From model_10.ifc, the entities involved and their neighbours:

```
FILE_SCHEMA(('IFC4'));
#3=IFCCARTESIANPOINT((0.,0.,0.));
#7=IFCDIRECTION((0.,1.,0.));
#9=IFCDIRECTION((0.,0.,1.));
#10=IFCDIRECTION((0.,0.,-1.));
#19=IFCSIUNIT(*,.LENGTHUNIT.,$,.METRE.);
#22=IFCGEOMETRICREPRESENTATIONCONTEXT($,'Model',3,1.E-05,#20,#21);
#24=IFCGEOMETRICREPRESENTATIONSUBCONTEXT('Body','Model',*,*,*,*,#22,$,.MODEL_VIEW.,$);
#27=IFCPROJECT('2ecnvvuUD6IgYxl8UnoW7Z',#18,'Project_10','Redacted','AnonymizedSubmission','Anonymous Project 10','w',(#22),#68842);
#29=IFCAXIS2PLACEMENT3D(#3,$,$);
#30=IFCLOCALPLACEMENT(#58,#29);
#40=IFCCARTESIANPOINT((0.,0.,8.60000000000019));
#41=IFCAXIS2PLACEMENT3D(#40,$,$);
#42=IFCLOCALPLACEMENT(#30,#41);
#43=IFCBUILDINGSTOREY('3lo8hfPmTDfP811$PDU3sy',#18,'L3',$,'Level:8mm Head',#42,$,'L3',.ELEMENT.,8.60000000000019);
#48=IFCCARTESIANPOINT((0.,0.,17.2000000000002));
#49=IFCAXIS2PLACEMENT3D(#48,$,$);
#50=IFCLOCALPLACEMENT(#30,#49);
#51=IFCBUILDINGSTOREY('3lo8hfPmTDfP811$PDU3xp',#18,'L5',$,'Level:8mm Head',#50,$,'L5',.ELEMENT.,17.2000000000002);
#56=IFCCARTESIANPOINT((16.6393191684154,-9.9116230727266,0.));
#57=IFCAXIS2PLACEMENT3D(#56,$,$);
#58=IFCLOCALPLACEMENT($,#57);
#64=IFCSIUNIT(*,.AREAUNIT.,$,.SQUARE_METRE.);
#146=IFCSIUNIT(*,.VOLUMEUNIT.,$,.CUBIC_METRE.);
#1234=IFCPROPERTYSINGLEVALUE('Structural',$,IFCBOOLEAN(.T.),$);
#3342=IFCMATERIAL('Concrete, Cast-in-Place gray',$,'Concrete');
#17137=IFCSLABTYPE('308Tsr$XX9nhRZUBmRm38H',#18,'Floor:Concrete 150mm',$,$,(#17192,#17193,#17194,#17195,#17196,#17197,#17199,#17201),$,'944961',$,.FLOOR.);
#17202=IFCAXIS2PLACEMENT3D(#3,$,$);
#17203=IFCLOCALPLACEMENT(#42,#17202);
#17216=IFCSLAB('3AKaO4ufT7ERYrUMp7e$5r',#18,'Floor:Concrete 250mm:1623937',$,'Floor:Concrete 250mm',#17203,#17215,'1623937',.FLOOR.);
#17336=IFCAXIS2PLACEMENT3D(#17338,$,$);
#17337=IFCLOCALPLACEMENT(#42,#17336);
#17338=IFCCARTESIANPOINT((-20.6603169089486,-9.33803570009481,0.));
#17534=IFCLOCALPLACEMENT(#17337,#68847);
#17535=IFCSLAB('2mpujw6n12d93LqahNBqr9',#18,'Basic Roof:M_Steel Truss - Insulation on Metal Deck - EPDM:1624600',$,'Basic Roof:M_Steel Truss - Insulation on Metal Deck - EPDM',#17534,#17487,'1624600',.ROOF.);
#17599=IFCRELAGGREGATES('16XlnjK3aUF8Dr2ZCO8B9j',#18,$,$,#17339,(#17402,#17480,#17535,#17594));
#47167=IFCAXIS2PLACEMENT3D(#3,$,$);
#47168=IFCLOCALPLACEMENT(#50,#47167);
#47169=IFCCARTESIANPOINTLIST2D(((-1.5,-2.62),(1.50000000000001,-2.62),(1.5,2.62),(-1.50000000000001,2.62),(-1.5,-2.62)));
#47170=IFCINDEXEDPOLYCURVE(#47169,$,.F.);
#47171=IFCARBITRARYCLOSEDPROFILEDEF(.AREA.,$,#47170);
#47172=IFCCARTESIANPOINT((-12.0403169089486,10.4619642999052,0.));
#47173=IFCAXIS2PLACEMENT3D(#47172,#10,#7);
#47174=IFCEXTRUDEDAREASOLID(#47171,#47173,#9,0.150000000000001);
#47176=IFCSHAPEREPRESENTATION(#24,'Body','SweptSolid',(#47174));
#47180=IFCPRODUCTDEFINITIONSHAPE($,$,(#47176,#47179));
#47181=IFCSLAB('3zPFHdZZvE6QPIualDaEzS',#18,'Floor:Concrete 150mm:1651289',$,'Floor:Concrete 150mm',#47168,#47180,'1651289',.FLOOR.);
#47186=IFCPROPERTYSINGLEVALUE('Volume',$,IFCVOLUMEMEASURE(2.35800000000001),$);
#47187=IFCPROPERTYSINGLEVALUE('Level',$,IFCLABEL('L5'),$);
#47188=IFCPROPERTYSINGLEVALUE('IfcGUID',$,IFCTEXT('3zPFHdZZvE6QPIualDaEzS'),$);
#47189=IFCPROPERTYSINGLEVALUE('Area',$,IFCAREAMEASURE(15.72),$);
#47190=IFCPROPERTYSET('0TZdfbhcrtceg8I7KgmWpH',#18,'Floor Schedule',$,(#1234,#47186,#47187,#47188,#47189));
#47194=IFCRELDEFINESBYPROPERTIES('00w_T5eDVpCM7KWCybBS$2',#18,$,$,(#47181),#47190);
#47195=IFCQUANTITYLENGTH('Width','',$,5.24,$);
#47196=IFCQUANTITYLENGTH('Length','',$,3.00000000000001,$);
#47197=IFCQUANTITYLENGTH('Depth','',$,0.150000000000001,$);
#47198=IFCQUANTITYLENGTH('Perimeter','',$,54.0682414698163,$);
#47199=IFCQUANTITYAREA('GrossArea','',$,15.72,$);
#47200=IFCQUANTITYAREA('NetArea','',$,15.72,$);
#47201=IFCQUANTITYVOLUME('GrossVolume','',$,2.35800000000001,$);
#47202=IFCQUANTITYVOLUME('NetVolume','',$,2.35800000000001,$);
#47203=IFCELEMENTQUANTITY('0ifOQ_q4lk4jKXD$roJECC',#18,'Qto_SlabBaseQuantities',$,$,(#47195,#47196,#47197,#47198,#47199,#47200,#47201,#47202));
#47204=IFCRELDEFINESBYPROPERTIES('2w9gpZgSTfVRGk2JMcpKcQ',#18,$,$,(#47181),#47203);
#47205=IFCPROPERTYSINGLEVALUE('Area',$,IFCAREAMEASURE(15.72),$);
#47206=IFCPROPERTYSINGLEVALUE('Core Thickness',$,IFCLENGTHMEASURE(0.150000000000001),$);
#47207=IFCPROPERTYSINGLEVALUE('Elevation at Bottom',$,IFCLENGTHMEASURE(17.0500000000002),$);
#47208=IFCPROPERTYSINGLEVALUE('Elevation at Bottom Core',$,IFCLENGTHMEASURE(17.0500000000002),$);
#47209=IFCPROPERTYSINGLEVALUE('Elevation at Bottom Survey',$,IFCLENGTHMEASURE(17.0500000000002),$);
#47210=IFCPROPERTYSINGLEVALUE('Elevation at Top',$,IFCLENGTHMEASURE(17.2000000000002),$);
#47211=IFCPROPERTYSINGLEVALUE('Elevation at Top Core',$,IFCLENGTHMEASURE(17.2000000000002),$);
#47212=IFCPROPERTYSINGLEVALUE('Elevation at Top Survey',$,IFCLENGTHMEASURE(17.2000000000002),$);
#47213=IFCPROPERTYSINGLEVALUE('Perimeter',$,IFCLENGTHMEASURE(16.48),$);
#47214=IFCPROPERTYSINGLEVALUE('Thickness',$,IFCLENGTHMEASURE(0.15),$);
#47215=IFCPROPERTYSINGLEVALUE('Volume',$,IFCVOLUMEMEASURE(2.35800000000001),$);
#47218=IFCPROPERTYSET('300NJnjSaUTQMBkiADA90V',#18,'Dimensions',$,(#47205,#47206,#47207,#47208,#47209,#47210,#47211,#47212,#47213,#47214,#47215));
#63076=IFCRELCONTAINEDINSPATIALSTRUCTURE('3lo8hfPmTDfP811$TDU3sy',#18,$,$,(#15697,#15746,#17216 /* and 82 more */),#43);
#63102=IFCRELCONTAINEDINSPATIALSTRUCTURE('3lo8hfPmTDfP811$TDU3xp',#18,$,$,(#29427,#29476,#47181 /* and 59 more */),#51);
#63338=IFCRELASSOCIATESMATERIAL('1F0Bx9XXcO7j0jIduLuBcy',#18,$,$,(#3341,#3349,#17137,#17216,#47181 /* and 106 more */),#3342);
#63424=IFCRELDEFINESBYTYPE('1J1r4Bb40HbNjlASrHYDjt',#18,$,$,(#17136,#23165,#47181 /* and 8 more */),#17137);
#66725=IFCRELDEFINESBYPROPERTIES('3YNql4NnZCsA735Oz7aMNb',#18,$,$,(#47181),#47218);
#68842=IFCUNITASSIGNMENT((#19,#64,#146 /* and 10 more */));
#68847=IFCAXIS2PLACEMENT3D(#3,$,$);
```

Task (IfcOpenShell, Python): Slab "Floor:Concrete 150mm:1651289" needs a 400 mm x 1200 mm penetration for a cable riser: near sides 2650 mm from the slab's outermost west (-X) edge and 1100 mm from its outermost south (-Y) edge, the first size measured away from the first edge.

```python
import numpy as np
import ifcopenshell
import ifcopenshell.api.feature
import ifcopenshell.api.geometry
import ifcopenshell.api.pset
import ifcopenshell.api.root
import ifcopenshell.geom
import ifcopenshell.util.element
import ifcopenshell.util.placement
import ifcopenshell.util.representation
import ifcopenshell.util.shape
import ifcopenshell.util.unit

model = ifcopenshell.open("model_10.ifc")
unit_scale = ifcopenshell.util.unit.calculate_unit_scale(model)
area_scale = ifcopenshell.util.unit.calculate_unit_scale(model, "AREAUNIT")
volume_scale = ifcopenshell.util.unit.calculate_unit_scale(model, "VOLUMEUNIT")
settings = ifcopenshell.geom.settings()


def volume(element):
    """Net volume in cubic metres, openings subtracted."""
    shape = ifcopenshell.geom.create_shape(settings, element)
    return ifcopenshell.util.shape.get_volume(shape.geometry)


slab = model.by_guid("3zPFHdZZvE6QPIualDaEzS")
before = volume(slab)

# Extent in the slab's own axes, in metres. The edges named are its -X and -Y sides.
slab_shape = ifcopenshell.geom.create_shape(settings, slab)
vertices = ifcopenshell.util.shape.get_vertices(slab_shape.geometry)
x_min, y_min, bottom = vertices.min(axis=0)
top = vertices[:, 2].max()

opening = ifcopenshell.api.root.create_entity(model, ifc_class="IfcOpeningElement", name="Cable riser opening", predefined_type="OPENING")
context = ifcopenshell.util.representation.get_context(model, "Model", "Body", "MODEL_VIEW")
width, depth = 0.4, 1.2
outline = [(0.0, 0.0), (width, 0.0), (width, depth), (0.0, depth), (0.0, 0.0)]
# Overshoot both faces by 50 mm so the cut is clean.
shape = ifcopenshell.api.geometry.add_slab_representation(
    model, context=context, depth=top - bottom + 0.1, polyline=outline
)
ifcopenshell.api.geometry.assign_representation(model, product=opening, representation=shape)

matrix = ifcopenshell.util.placement.get_local_placement(slab.ObjectPlacement)
matrix[:, 3] = matrix @ np.append(np.array([x_min + 2.65, y_min + 1.1, bottom - 0.05]) / unit_scale, 1.0)
ifcopenshell.api.geometry.edit_object_placement(model, product=opening, matrix=matrix, is_si=False)
ifcopenshell.api.feature.add_feature(model, feature=opening, element=slab)

after = volume(slab)

# Update the slab's stored quantities.
pset = model.by_id(ifcopenshell.util.element.get_pset(slab, "Floor Schedule", should_inherit=False)["id"])
ifcopenshell.api.pset.edit_pset(model, pset=pset, properties={
    "Volume": model.create_entity("IfcVolumeMeasure", after / volume_scale),
    "Area": model.create_entity("IfcAreaMeasure", after / (top - bottom) / area_scale),
})
qto = model.by_id(ifcopenshell.util.element.get_pset(slab, "Qto_SlabBaseQuantities", should_inherit=False)["id"])
ifcopenshell.api.pset.edit_qto(model, qto=qto, properties={
    "NetArea": after / (top - bottom) / area_scale,
    "NetVolume": after / volume_scale,
})
pset = model.by_id(ifcopenshell.util.element.get_pset(slab, "Dimensions", should_inherit=False)["id"])
ifcopenshell.api.pset.edit_pset(model, pset=pset, properties={
    "Area": model.create_entity("IfcAreaMeasure", after / (top - bottom) / area_scale),
    "Volume": model.create_entity("IfcVolumeMeasure", after / volume_scale),
})

print(f"slab volume {before:.3f} -> {after:.3f} m3")

model.write("model_10-out.ifc")
```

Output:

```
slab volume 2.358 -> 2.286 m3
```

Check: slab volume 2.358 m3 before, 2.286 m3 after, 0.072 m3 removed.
